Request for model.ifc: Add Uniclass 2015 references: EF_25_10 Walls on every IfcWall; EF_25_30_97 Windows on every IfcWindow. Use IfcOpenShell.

First a look at what the model holds.

```python
import ifcopenshell

model = ifcopenshell.open("model.ifc")
print(model.schema)
print("classifications:", [c.Name for c in model.by_type("IfcClassification")])
for ifc_class in ("IfcDoor", "IfcRoof", "IfcStair", "IfcWall", "IfcWindow"):
    print(ifc_class, len(model.by_type(ifc_class)))
```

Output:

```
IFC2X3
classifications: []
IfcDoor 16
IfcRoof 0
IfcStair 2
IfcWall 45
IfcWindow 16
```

```python
import ifcopenshell
import ifcopenshell.api.classification

model = ifcopenshell.open("model.ifc")

# IFC2X3 requires Source and Edition and has no link from the project to the system.
system = model.create_entity("IfcClassification", Source="NBS", Edition="2015", Name="Uniclass 2015")

codes = {
    "IfcWall": ("EF_25_10", "Walls"),
    "IfcWindow": ("EF_25_30_97", "Windows"),
}
for ifc_class, (code, name) in codes.items():
    products = model.by_type(ifc_class)
    ifcopenshell.api.classification.add_reference(
        model, products=products, classification=system, identification=code, name=name
    )
    print(code, len(products))

model.write("model_rev.ifc")
```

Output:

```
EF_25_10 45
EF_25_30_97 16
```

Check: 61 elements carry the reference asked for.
